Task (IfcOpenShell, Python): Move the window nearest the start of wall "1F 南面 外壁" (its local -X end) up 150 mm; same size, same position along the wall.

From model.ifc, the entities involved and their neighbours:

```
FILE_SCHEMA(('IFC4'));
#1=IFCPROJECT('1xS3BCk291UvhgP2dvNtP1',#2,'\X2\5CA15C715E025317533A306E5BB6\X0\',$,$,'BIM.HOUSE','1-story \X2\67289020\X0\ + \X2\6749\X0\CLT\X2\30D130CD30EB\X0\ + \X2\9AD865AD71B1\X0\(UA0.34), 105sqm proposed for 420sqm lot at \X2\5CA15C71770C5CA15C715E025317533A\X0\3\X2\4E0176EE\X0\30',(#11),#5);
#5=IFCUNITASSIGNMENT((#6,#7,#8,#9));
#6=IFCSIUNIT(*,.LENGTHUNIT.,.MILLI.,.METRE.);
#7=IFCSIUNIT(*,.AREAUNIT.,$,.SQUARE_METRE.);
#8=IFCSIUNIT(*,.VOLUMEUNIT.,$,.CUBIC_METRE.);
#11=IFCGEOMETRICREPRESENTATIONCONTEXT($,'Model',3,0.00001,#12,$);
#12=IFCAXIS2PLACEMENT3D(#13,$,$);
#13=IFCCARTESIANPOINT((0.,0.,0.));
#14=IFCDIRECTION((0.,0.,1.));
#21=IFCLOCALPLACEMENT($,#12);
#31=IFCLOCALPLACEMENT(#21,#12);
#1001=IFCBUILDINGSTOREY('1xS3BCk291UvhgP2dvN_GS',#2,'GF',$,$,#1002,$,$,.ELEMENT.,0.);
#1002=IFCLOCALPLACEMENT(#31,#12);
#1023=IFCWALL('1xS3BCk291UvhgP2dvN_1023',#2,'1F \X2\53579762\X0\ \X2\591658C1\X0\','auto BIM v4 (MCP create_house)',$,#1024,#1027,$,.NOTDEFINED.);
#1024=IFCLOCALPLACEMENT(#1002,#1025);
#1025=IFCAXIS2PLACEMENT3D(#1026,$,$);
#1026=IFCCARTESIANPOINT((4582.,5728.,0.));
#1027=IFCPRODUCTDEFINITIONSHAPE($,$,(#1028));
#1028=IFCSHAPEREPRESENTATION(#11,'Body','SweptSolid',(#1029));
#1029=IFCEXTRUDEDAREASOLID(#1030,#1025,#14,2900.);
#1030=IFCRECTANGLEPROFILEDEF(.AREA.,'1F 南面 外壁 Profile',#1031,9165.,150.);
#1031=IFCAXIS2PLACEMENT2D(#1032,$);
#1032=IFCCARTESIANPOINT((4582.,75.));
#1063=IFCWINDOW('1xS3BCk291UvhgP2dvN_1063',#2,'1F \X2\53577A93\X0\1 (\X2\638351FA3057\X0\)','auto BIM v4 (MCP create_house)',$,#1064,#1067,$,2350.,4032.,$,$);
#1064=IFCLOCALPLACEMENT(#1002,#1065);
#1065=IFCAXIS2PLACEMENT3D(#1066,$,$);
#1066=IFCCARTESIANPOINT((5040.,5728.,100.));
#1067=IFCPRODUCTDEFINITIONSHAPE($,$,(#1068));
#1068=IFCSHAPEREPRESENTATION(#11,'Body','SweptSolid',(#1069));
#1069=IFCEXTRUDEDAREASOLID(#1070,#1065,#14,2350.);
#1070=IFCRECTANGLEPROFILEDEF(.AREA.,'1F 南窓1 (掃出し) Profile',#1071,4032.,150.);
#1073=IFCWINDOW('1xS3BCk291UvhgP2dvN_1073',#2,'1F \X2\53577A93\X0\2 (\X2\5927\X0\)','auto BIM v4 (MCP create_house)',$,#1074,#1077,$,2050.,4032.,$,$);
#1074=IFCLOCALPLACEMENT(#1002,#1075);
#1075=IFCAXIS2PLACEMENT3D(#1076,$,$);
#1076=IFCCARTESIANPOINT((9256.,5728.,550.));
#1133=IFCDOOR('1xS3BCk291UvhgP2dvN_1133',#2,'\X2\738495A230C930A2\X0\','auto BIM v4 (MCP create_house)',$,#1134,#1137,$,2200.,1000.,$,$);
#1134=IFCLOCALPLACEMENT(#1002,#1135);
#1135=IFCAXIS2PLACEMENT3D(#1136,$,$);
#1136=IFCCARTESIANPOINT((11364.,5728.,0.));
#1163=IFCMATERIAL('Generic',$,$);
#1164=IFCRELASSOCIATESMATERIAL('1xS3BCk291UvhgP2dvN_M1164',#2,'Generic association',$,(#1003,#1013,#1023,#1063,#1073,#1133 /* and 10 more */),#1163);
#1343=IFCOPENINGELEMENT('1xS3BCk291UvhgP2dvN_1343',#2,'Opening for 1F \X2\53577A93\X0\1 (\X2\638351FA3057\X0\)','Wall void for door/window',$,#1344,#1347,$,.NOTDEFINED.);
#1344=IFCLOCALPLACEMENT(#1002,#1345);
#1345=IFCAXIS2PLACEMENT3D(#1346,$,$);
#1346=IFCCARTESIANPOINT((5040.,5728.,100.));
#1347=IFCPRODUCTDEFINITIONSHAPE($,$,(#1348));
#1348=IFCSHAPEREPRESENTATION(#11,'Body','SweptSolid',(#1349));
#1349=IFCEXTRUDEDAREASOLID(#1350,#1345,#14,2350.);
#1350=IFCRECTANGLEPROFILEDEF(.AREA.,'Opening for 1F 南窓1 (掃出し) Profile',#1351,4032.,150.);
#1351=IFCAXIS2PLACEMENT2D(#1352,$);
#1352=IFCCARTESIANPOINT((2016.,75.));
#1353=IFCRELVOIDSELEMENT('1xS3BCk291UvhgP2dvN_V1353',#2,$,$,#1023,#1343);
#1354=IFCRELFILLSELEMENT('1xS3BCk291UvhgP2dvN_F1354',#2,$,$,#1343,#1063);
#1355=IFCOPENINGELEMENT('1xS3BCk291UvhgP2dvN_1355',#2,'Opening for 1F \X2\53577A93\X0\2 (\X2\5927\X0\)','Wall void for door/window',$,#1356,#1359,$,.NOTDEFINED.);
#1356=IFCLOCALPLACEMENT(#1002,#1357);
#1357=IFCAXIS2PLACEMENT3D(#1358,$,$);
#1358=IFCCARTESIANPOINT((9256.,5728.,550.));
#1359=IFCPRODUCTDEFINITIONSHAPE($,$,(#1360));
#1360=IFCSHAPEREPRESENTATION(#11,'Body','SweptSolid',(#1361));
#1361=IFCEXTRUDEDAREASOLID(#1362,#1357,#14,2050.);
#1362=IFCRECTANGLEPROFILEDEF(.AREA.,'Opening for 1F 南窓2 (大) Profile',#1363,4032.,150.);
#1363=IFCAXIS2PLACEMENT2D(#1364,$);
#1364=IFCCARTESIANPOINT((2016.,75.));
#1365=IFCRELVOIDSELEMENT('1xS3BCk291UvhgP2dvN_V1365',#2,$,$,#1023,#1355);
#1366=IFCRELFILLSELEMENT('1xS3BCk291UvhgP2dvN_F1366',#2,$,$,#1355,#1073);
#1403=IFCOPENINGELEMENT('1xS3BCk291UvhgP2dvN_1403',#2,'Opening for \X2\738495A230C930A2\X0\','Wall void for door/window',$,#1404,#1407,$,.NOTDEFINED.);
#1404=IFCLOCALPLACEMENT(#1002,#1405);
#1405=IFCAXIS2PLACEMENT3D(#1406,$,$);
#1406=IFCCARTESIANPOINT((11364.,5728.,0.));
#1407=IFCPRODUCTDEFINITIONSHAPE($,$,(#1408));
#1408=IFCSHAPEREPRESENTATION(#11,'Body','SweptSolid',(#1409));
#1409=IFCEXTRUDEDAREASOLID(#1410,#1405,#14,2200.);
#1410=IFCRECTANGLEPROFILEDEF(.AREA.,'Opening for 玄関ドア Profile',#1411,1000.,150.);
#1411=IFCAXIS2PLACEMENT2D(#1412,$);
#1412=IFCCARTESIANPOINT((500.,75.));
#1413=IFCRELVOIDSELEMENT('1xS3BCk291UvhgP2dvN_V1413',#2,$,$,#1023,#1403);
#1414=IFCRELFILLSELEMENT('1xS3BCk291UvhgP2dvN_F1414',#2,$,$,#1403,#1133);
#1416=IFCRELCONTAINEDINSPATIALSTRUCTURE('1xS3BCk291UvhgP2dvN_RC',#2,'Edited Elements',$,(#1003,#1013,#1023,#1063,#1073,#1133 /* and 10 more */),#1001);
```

```python
import numpy as np
import ifcopenshell
import ifcopenshell.api.geometry
import ifcopenshell.util.placement
import ifcopenshell.util.unit

model = ifcopenshell.open("model.ifc")
unit_scale = ifcopenshell.util.unit.calculate_unit_scale(model)

window = model.by_guid("1xS3BCk291UvhgP2dvN_1063")
opening = window.FillsVoids[0].RelatingOpeningElement
dz = 0.15 / unit_scale

shift = np.array([0.0, 0.0, dz])
# The window is not placed relative to its opening, so move both.
for product in (opening, window):
    matrix = ifcopenshell.util.placement.get_local_placement(product.ObjectPlacement)
    matrix[:3, 3] += shift
    ifcopenshell.api.geometry.edit_object_placement(model, product=product, matrix=matrix, is_si=False)

print(f"moved by {dz * unit_scale:+.3f} m")

model.write("model_v2.ifc")
```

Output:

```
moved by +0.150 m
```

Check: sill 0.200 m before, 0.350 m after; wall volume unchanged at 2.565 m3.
